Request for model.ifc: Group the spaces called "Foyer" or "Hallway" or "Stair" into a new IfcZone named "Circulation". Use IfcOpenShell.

First a look at what the model holds.

```python
import ifcopenshell

model = ifcopenshell.open("model.ifc")
print(model.schema)
seen = {}
for space in model.by_type("IfcSpace"):
    seen[space.LongName] = seen.get(space.LongName, 0) + 1
for name, count in sorted(seen.items(), key=str):
    print(count, "x", name)
print("zones:", [z.Name for z in model.by_type("IfcZone")][:20])
```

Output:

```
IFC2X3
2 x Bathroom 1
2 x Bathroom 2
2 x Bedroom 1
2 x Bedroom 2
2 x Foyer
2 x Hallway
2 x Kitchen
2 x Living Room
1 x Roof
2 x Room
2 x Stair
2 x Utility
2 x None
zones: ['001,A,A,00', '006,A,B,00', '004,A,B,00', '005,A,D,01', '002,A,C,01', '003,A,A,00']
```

```python
import ifcopenshell
import ifcopenshell.api.group
import ifcopenshell.api.root

model = ifcopenshell.open("model.ifc")

names = {"Foyer", "Hallway", "Stair"}
spaces = [s for s in model.by_type("IfcSpace") if s.LongName in names]

zone = ifcopenshell.api.root.create_entity(model, ifc_class="IfcZone", name="Circulation")
ifcopenshell.api.group.assign_group(model, products=spaces, group=zone)
print(len(spaces), "spaces in", zone.Name)

model.write("model_v2.ifc")
```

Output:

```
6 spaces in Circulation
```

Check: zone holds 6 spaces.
